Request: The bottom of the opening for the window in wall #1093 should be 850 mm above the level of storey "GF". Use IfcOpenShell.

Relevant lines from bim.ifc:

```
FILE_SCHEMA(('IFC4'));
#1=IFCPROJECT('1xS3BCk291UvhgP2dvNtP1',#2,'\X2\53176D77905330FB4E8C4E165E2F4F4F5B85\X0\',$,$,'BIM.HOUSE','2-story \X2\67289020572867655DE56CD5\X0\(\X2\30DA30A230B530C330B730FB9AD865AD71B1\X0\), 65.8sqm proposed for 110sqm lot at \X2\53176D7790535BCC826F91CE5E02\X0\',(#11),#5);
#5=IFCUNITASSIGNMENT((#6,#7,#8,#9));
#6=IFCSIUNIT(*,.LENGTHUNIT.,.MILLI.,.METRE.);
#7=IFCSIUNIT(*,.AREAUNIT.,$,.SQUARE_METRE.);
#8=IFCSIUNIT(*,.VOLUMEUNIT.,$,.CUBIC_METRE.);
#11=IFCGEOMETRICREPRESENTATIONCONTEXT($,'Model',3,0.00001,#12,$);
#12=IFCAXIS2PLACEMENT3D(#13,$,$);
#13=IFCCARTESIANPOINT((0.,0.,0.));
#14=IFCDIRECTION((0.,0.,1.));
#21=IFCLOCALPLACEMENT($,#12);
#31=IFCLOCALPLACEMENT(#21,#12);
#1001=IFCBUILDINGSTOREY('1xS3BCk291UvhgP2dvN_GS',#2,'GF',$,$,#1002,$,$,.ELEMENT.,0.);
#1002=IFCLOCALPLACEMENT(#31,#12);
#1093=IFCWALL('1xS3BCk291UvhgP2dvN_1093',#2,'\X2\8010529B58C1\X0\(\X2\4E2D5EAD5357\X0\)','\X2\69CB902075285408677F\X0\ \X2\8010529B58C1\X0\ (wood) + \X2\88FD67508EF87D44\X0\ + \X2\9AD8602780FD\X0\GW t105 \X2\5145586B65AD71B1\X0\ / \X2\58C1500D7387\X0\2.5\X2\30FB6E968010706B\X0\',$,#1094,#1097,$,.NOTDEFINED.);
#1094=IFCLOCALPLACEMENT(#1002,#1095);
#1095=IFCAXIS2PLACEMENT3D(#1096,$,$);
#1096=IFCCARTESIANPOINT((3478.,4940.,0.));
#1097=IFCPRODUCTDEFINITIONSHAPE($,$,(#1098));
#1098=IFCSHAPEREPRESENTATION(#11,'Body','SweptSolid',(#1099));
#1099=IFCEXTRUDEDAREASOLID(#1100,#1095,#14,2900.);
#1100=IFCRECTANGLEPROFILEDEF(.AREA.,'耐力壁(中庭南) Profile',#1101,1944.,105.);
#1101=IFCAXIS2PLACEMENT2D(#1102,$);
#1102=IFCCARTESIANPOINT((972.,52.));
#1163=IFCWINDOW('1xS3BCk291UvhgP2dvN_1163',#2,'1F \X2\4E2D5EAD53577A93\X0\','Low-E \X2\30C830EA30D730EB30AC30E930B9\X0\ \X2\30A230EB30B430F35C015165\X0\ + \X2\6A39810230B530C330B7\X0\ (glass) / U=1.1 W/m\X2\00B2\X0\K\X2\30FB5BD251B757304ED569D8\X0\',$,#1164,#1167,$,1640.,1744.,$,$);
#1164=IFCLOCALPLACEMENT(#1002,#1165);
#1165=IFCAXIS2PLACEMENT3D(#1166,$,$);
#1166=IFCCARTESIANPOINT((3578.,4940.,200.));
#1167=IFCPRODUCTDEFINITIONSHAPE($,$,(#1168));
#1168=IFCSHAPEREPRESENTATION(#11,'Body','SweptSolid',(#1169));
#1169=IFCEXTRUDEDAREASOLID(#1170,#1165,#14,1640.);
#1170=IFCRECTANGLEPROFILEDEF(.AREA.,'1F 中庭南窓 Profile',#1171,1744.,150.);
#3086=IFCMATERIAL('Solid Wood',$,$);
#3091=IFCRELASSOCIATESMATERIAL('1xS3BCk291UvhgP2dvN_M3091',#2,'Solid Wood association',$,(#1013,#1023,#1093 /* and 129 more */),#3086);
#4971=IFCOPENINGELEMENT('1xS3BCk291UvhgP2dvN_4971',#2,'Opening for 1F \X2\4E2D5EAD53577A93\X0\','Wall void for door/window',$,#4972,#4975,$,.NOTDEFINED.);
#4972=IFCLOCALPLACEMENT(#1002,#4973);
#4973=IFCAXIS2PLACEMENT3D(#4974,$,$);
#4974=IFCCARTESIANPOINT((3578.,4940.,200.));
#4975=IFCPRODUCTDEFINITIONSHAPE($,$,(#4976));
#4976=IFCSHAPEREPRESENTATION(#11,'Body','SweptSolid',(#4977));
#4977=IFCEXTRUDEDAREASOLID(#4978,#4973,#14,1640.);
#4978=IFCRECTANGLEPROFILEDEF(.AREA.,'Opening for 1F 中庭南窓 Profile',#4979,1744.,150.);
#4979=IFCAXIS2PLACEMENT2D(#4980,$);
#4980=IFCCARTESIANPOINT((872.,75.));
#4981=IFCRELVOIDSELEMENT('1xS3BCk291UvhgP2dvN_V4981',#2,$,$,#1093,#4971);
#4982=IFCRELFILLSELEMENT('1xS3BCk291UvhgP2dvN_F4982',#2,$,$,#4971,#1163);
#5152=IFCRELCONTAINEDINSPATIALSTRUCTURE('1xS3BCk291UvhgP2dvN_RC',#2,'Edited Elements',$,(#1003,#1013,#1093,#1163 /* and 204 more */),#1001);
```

```python
import numpy as np
import ifcopenshell
import ifcopenshell.api.geometry
import ifcopenshell.geom
import ifcopenshell.util.element
import ifcopenshell.util.placement
import ifcopenshell.util.shape
import ifcopenshell.util.unit

model = ifcopenshell.open("bim.ifc")
unit_scale = ifcopenshell.util.unit.calculate_unit_scale(model)

window = model.by_guid("1xS3BCk291UvhgP2dvN_1163")
opening = window.FillsVoids[0].RelatingOpeningElement
storey = ifcopenshell.util.element.get_container(window, ifc_class="IfcBuildingStorey")
level = ifcopenshell.util.placement.get_local_placement(storey.ObjectPlacement)[2, 3]

# The opening's origin need not be at the sill, so measure its lowest point.
shape = ifcopenshell.geom.create_shape(ifcopenshell.geom.settings(), opening)
bottom = ifcopenshell.util.shape.get_shape_bottom_elevation(shape, shape.geometry) / unit_scale
dz = level + 850.0 - bottom

shift = np.array([0.0, 0.0, dz])
# The window is not placed relative to its opening, so move both.
for product in (opening, window):
    matrix = ifcopenshell.util.placement.get_local_placement(product.ObjectPlacement)
    matrix[:3, 3] += shift
    ifcopenshell.api.geometry.edit_object_placement(model, product=product, matrix=matrix, is_si=False)

print(f"moved by {dz * unit_scale:+.3f} m")

model.write("bim_rev.ifc")
```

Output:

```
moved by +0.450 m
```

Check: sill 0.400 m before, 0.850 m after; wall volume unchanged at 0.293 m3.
